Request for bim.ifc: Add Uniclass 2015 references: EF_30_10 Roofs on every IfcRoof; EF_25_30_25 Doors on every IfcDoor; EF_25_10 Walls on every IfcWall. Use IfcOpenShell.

First a look at what the model holds.

```python
import ifcopenshell

model = ifcopenshell.open("bim.ifc")
print(model.schema)
print("classifications:", [c.Name for c in model.by_type("IfcClassification")])
for ifc_class in ("IfcDoor", "IfcRoof", "IfcStair", "IfcWall", "IfcWindow"):
    print(ifc_class, len(model.by_type(ifc_class)))
```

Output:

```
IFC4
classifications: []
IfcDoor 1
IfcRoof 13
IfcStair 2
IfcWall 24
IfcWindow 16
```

```python
import ifcopenshell
import ifcopenshell.api.classification

model = ifcopenshell.open("bim.ifc")

system = ifcopenshell.api.classification.add_classification(model, classification="Uniclass 2015")

codes = {
    "IfcRoof": ("EF_30_10", "Roofs"),
    "IfcDoor": ("EF_25_30_25", "Doors"),
    "IfcWall": ("EF_25_10", "Walls"),
}
for ifc_class, (code, name) in codes.items():
    products = model.by_type(ifc_class)
    ifcopenshell.api.classification.add_reference(
        model, products=products, classification=system, identification=code, name=name
    )
    print(code, len(products))

model.write("bim-out.ifc")
```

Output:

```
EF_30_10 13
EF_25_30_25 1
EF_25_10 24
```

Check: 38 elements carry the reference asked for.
